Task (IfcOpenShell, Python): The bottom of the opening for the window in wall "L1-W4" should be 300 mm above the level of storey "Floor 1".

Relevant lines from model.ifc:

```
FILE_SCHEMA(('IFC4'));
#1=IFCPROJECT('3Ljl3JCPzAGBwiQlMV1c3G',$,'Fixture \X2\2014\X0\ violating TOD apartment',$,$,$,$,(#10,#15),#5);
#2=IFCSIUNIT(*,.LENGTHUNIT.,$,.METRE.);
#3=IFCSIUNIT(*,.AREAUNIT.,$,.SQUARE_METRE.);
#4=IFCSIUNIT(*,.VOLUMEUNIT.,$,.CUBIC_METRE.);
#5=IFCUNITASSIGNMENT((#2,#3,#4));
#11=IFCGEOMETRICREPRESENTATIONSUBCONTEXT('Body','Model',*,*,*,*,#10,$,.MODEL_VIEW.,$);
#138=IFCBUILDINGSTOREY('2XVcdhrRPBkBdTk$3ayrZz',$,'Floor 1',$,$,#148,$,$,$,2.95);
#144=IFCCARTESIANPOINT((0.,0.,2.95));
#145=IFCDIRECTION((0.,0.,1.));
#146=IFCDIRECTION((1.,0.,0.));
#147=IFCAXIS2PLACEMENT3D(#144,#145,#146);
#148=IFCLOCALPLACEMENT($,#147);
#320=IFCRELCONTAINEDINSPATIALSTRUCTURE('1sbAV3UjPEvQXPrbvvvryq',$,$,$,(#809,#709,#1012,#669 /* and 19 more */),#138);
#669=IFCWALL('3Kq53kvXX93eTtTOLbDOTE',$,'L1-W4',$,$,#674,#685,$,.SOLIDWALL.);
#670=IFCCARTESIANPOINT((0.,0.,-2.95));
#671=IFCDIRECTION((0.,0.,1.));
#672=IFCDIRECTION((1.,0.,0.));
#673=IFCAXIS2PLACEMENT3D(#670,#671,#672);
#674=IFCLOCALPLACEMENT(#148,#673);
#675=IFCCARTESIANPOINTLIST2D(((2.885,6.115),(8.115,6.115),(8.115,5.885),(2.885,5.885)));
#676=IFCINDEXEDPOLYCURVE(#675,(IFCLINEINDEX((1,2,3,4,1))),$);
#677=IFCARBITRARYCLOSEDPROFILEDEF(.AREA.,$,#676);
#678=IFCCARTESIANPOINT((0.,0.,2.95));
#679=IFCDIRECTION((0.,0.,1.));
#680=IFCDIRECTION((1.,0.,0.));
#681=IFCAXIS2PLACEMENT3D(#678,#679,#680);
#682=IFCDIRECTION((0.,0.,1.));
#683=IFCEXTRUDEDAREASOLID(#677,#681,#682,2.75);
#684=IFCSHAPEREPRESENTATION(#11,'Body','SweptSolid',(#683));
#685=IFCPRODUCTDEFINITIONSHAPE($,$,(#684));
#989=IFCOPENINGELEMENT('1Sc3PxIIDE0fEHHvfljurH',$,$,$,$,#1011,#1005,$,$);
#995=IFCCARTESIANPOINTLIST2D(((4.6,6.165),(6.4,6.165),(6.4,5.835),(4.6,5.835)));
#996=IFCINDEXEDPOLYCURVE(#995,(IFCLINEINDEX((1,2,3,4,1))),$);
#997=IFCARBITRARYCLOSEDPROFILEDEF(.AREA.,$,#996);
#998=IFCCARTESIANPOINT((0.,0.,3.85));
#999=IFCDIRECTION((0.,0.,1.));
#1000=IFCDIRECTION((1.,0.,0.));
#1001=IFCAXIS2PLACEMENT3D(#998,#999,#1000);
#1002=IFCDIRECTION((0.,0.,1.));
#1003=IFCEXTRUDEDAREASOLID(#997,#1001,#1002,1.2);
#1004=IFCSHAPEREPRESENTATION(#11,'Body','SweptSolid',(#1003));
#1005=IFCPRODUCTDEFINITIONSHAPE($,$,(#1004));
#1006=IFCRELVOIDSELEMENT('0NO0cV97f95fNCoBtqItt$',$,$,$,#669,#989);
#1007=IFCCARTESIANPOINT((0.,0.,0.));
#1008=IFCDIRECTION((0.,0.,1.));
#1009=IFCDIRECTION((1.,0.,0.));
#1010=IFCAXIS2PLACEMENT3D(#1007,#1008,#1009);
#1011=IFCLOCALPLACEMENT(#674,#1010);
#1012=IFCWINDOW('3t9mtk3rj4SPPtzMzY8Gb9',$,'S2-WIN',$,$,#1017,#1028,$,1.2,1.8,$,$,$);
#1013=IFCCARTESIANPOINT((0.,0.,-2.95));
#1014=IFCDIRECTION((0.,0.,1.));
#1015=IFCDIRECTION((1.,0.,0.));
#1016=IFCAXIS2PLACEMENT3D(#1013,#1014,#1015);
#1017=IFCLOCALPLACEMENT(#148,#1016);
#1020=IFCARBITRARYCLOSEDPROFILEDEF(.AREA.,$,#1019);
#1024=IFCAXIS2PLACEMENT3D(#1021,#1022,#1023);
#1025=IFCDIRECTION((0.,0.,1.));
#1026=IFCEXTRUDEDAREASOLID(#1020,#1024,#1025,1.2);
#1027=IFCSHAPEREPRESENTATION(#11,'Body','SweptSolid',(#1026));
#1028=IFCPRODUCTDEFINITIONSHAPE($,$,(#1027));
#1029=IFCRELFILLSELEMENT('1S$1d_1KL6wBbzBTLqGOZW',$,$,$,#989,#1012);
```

```python
import numpy as np
import ifcopenshell
import ifcopenshell.api.geometry
import ifcopenshell.geom
import ifcopenshell.util.element
import ifcopenshell.util.placement
import ifcopenshell.util.shape
import ifcopenshell.util.unit

model = ifcopenshell.open("model.ifc")
unit_scale = ifcopenshell.util.unit.calculate_unit_scale(model)

window = model.by_guid("3t9mtk3rj4SPPtzMzY8Gb9")
opening = window.FillsVoids[0].RelatingOpeningElement
storey = ifcopenshell.util.element.get_container(window, ifc_class="IfcBuildingStorey")
level = ifcopenshell.util.placement.get_local_placement(storey.ObjectPlacement)[2, 3]

# The opening's origin need not be at the sill, so measure its lowest point.
shape = ifcopenshell.geom.create_shape(ifcopenshell.geom.settings(), opening)
bottom = ifcopenshell.util.shape.get_shape_bottom_elevation(shape, shape.geometry) / unit_scale
dz = level + 0.3 - bottom

shift = np.array([0.0, 0.0, dz])
# The window is not placed relative to its opening, so move both.
for product in (opening, window):
    matrix = ifcopenshell.util.placement.get_local_placement(product.ObjectPlacement)
    matrix[:3, 3] += shift
    ifcopenshell.api.geometry.edit_object_placement(model, product=product, matrix=matrix, is_si=False)

print(f"moved by {dz * unit_scale:+.3f} m")

model.write("model_rev.ifc")
```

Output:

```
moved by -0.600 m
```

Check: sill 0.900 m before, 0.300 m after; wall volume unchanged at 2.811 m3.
